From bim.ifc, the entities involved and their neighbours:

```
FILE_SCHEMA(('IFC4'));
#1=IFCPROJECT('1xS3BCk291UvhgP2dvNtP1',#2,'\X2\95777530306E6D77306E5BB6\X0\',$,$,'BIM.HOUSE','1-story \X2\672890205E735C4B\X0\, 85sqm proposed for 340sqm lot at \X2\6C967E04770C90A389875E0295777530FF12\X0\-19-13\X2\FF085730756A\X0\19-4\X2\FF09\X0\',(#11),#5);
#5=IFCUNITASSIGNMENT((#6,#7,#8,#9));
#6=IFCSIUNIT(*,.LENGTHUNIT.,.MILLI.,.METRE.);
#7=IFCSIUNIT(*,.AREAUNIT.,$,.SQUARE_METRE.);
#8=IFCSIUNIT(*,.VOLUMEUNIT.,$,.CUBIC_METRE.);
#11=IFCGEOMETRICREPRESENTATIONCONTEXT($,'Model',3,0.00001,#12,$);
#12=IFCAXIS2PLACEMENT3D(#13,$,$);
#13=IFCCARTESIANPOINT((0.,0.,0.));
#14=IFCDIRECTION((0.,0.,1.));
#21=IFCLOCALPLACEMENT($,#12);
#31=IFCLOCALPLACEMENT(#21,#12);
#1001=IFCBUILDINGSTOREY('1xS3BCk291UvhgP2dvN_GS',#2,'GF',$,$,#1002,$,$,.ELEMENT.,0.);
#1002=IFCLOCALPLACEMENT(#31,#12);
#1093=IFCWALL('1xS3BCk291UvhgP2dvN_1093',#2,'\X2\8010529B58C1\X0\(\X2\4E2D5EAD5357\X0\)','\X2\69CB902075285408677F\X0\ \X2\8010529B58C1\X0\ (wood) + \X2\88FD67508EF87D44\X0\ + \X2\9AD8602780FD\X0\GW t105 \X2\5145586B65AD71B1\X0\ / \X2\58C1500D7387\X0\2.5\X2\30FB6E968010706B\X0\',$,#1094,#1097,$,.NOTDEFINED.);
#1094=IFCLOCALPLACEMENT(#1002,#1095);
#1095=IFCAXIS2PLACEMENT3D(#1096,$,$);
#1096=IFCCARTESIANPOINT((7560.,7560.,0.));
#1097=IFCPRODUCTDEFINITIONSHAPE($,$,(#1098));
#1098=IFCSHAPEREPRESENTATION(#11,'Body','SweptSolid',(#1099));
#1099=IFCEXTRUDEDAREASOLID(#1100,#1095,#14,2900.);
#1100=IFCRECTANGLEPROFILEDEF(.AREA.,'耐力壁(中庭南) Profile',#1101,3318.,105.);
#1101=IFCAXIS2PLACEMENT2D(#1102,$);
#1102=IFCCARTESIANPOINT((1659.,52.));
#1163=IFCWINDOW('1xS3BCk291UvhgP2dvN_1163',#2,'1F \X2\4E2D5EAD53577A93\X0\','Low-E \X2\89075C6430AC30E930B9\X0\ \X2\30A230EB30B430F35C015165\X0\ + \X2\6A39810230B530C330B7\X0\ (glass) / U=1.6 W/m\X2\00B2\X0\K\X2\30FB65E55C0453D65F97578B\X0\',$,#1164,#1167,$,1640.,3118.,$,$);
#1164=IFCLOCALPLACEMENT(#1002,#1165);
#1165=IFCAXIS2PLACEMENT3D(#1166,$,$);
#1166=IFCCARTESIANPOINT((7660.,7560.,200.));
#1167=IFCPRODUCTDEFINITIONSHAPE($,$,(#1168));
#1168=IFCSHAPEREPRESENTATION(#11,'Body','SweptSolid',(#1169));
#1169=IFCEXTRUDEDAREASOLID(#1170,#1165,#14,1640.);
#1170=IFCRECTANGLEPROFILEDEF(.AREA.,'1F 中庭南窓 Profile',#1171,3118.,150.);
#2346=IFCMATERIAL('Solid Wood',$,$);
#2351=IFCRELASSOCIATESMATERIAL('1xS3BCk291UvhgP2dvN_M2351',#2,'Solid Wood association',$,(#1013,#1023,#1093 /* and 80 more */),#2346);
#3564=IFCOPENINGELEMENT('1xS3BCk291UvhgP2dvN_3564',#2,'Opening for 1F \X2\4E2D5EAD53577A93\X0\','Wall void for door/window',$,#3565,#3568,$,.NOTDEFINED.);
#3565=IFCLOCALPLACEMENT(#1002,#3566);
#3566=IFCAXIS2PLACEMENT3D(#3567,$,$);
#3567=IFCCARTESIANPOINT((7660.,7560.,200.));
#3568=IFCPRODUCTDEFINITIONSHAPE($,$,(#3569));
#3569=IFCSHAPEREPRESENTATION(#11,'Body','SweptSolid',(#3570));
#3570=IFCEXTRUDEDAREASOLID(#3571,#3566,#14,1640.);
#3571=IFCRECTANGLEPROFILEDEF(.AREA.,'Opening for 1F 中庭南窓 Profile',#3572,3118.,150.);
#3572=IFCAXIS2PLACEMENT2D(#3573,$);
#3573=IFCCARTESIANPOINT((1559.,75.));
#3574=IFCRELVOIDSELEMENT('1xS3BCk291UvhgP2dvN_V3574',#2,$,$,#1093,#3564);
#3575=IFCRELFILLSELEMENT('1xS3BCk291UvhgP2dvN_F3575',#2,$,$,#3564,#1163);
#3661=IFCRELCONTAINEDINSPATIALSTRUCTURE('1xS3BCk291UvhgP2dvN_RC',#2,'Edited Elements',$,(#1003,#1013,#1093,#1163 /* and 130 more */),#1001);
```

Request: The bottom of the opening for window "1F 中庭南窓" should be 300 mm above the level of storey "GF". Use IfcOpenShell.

```python
import numpy as np
import ifcopenshell
import ifcopenshell.api.geometry
import ifcopenshell.geom
import ifcopenshell.util.element
import ifcopenshell.util.placement
import ifcopenshell.util.shape
import ifcopenshell.util.unit

model = ifcopenshell.open("bim.ifc")
unit_scale = ifcopenshell.util.unit.calculate_unit_scale(model)

window = model.by_guid("1xS3BCk291UvhgP2dvN_1163")
opening = window.FillsVoids[0].RelatingOpeningElement
storey = ifcopenshell.util.element.get_container(window, ifc_class="IfcBuildingStorey")
level = ifcopenshell.util.placement.get_local_placement(storey.ObjectPlacement)[2, 3]

# The opening's origin need not be at the sill, so measure its lowest point.
shape = ifcopenshell.geom.create_shape(ifcopenshell.geom.settings(), opening)
bottom = ifcopenshell.util.shape.get_shape_bottom_elevation(shape, shape.geometry) / unit_scale
dz = level + 0.3 / unit_scale - bottom

shift = np.array([0.0, 0.0, dz])
# The window is not placed relative to its opening, so move both.
for product in (opening, window):
    matrix = ifcopenshell.util.placement.get_local_placement(product.ObjectPlacement)
    matrix[:3, 3] += shift
    ifcopenshell.api.geometry.edit_object_placement(model, product=product, matrix=matrix, is_si=False)

print(f"moved by {dz * unit_scale:+.3f} m")

model.write("bim_rev.ifc")
```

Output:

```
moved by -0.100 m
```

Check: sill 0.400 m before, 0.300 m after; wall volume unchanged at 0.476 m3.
